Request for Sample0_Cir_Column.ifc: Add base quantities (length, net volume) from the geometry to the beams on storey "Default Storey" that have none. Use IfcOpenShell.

First a look at what the model holds.

```python
import ifcopenshell
import ifcopenshell.util.element
import ifcopenshell.util.unit

model = ifcopenshell.open("Sample0_Cir_Column.ifc")
print(model.schema)
for unit_type in ("LENGTHUNIT", "AREAUNIT", "VOLUMEUNIT"):
    print(unit_type, ifcopenshell.util.unit.calculate_unit_scale(model, unit_type))
storey = next(s for s in model.by_type("IfcBuildingStorey") if s.Name == "Default Storey")
beams = [e for e in ifcopenshell.util.element.get_decomposition(storey) if e.is_a("IfcBeam")]
for e in sorted(beams, key=lambda e: e.id()):
    print(e.id(), e.is_a(), e.Name, list(ifcopenshell.util.element.get_psets(e, qtos_only=True)), sep=" | ")
```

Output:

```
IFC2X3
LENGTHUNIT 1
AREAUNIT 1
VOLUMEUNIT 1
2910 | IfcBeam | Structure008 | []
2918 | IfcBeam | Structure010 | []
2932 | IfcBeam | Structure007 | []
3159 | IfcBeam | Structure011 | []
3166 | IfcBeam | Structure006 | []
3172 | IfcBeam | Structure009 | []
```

```python
import ifcopenshell
import ifcopenshell.api.pset
import ifcopenshell.geom
import ifcopenshell.util.element
import ifcopenshell.util.shape
import ifcopenshell.util.unit

model = ifcopenshell.open("Sample0_Cir_Column.ifc")
unit_scale = ifcopenshell.util.unit.calculate_unit_scale(model)
volume_scale = ifcopenshell.util.unit.calculate_unit_scale(model, "VOLUMEUNIT")
settings = ifcopenshell.geom.settings()

storey = next(s for s in model.by_type("IfcBuildingStorey") if s.Name == "Default Storey")
beams = [e for e in ifcopenshell.util.element.get_decomposition(storey) if e.is_a("IfcBeam")]

for e in sorted(beams, key=lambda e: e.id()):
    if ifcopenshell.util.element.get_psets(e, qtos_only=True, should_inherit=False):
        continue
    # Geometry comes back in metres, in the element's own axes.
    shape = ifcopenshell.geom.create_shape(settings, e)
    values = {
        "Length": ifcopenshell.util.shape.get_max_xyz(shape.geometry) / unit_scale,
        "NetVolume": ifcopenshell.util.shape.get_volume(shape.geometry) / volume_scale,
    }
    qto = ifcopenshell.api.pset.add_qto(model, product=e, name="BaseQuantities")
    ifcopenshell.api.pset.edit_qto(model, qto=qto, properties=values)
    print(e.id(), {k: round(v, 3) for k, v in values.items()})

model.write("Sample0_Cir_Column_rev.ifc")
```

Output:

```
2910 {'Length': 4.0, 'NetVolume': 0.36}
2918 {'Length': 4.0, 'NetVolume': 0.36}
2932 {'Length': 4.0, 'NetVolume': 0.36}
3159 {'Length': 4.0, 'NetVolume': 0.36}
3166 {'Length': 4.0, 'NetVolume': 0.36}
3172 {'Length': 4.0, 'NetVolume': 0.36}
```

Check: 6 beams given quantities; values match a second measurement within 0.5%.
